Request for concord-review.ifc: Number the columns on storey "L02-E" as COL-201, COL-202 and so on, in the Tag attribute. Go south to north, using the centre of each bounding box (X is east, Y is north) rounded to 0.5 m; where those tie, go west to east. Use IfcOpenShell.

First a look at what the model holds.

```python
import ifcopenshell
import ifcopenshell.util.element
import ifcopenshell.util.placement

model = ifcopenshell.open("concord-review.ifc")
print(model.schema)
storey = next(s for s in model.by_type("IfcBuildingStorey") if s.Name == "L02-E")
columns = [e for e in ifcopenshell.util.element.get_decomposition(storey) if e.is_a("IfcColumn")]
for e in sorted(columns, key=lambda e: e.id()):
    origin = ifcopenshell.util.placement.get_local_placement(e.ObjectPlacement)[:3, 3]
    print(e.id(), e.Tag, e.Name, origin.round(2) + 0.0, sep=" | ")
```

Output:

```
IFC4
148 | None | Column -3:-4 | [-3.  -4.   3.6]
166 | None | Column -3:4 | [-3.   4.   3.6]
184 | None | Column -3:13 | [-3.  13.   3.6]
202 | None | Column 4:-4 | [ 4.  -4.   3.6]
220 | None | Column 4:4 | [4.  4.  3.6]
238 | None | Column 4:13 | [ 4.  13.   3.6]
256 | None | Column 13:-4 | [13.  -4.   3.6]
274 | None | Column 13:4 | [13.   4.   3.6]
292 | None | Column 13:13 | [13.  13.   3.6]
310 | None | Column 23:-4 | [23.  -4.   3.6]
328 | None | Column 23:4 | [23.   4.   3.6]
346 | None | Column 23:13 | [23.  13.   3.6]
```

```python
import ifcopenshell
import ifcopenshell.geom
import ifcopenshell.util.element
import ifcopenshell.util.shape

model = ifcopenshell.open("concord-review.ifc")
settings = ifcopenshell.geom.settings()
settings.set("use-world-coords", True)


def centre(element):
    shape = ifcopenshell.geom.create_shape(settings, element)
    return ifcopenshell.util.shape.get_bbox_centroid(shape.geometry)


storey = next(s for s in model.by_type("IfcBuildingStorey") if s.Name == "L02-E")
columns = [e for e in ifcopenshell.util.element.get_decomposition(storey) if e.is_a("IfcColumn")]

# Insertion points can sit at a corner or the storey origin, so sort by the geometry (in metres).
centres = {e: centre(e) for e in columns}
columns.sort(key=lambda e: (round(centres[e][1] / 0.5), centres[e][0]))

for i, e in enumerate(columns, start=1):
    number = f"COL-2{i:02d}"
    e.Tag = number
    print(e.id(), number)

model.write("concord-review_updated.ifc")
```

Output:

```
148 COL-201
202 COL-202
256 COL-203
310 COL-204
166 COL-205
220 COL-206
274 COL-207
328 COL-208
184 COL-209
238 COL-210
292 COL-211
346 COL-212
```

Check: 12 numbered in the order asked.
